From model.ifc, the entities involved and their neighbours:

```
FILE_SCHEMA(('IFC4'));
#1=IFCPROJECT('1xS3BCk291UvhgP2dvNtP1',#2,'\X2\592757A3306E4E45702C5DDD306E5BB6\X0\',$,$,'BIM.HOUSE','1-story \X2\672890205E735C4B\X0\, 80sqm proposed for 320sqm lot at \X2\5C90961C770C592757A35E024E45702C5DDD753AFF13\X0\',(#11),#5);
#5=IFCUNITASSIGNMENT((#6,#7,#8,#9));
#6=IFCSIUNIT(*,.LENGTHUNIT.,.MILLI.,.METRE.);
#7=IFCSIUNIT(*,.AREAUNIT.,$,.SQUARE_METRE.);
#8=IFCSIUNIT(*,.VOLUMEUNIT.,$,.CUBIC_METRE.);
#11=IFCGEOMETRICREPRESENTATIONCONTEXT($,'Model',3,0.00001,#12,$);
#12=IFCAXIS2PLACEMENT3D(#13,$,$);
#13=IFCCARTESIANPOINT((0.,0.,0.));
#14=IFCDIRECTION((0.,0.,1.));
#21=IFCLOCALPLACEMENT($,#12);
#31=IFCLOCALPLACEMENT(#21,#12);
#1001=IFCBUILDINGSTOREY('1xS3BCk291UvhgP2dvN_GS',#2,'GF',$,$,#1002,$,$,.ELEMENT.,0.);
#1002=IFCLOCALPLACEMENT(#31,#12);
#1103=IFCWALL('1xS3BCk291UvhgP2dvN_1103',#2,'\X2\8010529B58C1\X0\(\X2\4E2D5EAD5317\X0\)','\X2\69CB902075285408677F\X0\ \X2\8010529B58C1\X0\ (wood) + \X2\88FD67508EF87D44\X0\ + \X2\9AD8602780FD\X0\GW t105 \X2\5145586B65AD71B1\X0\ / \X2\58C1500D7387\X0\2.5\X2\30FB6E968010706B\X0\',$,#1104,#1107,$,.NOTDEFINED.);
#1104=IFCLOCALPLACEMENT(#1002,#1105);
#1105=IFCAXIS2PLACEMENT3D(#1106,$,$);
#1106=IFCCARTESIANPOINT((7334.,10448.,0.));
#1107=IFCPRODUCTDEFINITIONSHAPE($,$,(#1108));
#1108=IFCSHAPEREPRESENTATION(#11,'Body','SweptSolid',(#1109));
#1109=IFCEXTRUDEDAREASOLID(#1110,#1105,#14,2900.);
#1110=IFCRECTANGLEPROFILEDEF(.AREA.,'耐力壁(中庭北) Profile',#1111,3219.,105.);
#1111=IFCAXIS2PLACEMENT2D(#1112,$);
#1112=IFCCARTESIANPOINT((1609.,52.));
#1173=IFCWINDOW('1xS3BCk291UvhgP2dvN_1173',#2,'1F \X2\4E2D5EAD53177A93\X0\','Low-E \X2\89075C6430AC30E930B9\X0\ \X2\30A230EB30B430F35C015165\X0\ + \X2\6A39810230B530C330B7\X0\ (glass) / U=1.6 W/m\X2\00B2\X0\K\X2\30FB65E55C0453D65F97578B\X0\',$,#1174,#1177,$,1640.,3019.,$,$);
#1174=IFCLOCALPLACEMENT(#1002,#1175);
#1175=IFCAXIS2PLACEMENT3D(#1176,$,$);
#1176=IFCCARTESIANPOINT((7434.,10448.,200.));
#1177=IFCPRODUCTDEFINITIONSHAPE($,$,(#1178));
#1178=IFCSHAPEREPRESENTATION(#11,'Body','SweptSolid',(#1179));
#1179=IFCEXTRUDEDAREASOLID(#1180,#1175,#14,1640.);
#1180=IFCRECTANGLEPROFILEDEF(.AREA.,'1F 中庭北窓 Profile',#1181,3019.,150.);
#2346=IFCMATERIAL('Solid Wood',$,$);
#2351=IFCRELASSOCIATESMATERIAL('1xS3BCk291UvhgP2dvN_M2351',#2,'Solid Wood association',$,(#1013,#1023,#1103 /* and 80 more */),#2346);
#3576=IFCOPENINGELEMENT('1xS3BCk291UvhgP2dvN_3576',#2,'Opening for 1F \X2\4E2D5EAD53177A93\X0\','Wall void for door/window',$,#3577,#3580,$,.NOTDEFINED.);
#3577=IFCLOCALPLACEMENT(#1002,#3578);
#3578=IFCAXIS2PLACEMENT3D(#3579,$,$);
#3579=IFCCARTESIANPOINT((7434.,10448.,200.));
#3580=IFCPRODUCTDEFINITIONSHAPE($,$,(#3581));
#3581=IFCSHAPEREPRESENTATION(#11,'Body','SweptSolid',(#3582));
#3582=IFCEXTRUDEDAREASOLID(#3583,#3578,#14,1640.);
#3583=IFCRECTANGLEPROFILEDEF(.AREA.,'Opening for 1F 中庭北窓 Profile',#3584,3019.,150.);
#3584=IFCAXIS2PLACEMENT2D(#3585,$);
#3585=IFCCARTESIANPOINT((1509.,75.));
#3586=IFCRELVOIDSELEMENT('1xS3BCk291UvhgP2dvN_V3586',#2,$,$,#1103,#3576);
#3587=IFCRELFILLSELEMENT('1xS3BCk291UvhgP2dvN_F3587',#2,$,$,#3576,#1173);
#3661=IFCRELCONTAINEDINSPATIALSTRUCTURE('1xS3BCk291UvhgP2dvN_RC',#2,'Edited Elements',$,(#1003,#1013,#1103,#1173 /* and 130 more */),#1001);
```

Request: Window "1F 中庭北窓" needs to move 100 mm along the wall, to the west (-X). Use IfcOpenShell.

```python
import ifcopenshell
import ifcopenshell.api.geometry
import ifcopenshell.util.placement
import ifcopenshell.util.unit

model = ifcopenshell.open("model.ifc")
unit_scale = ifcopenshell.util.unit.calculate_unit_scale(model)

window = model.by_guid("1xS3BCk291UvhgP2dvN_1173")
opening = window.FillsVoids[0].RelatingOpeningElement
wall = opening.VoidsElements[0].RelatingBuildingElement

wall_matrix = ifcopenshell.util.placement.get_local_placement(wall.ObjectPlacement)
shift = wall_matrix[:3, 0] * -0.1 / unit_scale
before = ifcopenshell.util.placement.get_local_placement(window.ObjectPlacement)[:3, 3].copy()

# The window is not placed relative to its opening, so move both.
for product in (opening, window):
    matrix = ifcopenshell.util.placement.get_local_placement(product.ObjectPlacement)
    matrix[:3, 3] += shift
    ifcopenshell.api.geometry.edit_object_placement(model, product=product, matrix=matrix, is_si=False)

after = ifcopenshell.util.placement.get_local_placement(window.ObjectPlacement)[:3, 3]
print("window moved by", (after - before).round(3) + 0.0)

model.write("model_rev.ifc")
```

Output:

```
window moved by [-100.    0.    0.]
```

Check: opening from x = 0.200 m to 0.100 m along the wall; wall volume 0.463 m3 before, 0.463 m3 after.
